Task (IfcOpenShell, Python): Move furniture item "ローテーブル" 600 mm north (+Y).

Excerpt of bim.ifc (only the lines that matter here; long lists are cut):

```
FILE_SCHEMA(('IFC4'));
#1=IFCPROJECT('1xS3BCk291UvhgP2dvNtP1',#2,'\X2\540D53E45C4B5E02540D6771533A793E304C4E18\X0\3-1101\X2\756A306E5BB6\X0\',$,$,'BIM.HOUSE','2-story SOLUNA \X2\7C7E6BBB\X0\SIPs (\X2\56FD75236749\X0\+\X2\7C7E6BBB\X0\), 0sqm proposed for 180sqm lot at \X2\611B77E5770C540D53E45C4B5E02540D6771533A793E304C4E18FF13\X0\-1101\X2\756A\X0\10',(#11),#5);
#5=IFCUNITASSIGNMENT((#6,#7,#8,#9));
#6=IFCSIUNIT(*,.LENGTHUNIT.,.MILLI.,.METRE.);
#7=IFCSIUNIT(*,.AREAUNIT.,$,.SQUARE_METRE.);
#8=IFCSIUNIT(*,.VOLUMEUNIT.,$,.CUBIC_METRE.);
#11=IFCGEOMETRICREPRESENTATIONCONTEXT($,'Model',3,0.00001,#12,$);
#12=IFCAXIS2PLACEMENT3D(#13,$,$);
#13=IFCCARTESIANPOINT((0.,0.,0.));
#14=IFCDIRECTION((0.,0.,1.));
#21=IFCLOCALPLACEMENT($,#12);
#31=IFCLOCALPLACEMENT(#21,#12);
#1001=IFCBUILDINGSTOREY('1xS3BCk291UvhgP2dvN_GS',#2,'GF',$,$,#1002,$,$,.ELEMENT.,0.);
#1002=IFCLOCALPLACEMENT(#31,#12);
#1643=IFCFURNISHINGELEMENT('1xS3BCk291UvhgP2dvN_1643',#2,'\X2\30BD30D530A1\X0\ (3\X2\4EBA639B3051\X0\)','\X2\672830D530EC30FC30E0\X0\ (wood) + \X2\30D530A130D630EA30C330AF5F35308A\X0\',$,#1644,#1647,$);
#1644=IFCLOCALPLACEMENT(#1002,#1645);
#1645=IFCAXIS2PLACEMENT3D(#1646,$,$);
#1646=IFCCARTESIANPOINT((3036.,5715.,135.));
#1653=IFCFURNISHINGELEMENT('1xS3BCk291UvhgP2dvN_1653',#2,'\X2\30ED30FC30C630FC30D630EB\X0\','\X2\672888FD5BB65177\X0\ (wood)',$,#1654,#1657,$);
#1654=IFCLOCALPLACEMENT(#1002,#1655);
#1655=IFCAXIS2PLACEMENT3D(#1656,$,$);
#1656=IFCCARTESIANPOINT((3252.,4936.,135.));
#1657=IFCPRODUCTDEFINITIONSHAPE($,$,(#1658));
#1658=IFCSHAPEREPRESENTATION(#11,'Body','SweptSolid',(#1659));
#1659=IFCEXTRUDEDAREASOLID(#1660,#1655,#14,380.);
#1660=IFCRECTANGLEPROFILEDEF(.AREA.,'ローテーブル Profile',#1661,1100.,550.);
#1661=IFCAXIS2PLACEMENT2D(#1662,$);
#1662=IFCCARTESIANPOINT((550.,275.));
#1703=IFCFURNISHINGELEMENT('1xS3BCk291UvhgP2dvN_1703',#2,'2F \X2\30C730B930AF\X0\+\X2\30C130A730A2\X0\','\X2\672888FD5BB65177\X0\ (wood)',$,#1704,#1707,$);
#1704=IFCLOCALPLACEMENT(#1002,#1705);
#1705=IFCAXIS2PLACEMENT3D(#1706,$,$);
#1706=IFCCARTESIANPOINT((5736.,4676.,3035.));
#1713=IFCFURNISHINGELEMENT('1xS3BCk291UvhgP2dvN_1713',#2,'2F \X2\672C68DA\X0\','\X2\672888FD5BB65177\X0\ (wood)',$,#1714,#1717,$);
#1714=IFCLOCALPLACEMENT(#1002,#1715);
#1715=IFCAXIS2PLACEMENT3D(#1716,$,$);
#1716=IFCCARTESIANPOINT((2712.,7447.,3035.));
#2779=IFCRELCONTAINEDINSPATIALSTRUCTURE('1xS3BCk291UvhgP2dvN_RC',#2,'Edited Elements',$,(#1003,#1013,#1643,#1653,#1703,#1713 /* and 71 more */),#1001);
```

```python
import ifcopenshell
import ifcopenshell.api.geometry
import ifcopenshell.util.placement

model = ifcopenshell.open("bim.ifc")

item = model.by_id(1653)
matrix = ifcopenshell.util.placement.get_local_placement(item.ObjectPlacement)
matrix[1, 3] += 600.0
ifcopenshell.api.geometry.edit_object_placement(model, product=item, matrix=matrix, is_si=False)

print(ifcopenshell.util.placement.get_local_placement(item.ObjectPlacement).round(3) + 0.0)

model.write("bim-out.ifc")
```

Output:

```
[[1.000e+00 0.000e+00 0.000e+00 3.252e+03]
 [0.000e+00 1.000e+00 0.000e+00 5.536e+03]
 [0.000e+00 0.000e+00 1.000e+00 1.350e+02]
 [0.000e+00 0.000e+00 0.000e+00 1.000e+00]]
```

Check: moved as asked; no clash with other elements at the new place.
